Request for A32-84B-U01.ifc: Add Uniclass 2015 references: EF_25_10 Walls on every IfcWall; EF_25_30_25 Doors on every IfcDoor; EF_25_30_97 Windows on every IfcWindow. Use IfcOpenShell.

First a look at what the model holds.

```python
import ifcopenshell

model = ifcopenshell.open("A32-84B-U01.ifc")
print(model.schema)
print("classifications:", [c.Name for c in model.by_type("IfcClassification")])
for ifc_class in ("IfcDoor", "IfcRoof", "IfcStair", "IfcWall", "IfcWindow"):
    print(ifc_class, len(model.by_type(ifc_class)))
```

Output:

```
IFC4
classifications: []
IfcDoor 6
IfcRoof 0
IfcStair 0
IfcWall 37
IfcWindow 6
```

```python
import ifcopenshell
import ifcopenshell.api.classification

model = ifcopenshell.open("A32-84B-U01.ifc")

system = ifcopenshell.api.classification.add_classification(model, classification="Uniclass 2015")

codes = {
    "IfcWall": ("EF_25_10", "Walls"),
    "IfcDoor": ("EF_25_30_25", "Doors"),
    "IfcWindow": ("EF_25_30_97", "Windows"),
}
for ifc_class, (code, name) in codes.items():
    products = model.by_type(ifc_class)
    ifcopenshell.api.classification.add_reference(
        model, products=products, classification=system, identification=code, name=name
    )
    print(code, len(products))

model.write("A32-84B-U01_v2.ifc")
```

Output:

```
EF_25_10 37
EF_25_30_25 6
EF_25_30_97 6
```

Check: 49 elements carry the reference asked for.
